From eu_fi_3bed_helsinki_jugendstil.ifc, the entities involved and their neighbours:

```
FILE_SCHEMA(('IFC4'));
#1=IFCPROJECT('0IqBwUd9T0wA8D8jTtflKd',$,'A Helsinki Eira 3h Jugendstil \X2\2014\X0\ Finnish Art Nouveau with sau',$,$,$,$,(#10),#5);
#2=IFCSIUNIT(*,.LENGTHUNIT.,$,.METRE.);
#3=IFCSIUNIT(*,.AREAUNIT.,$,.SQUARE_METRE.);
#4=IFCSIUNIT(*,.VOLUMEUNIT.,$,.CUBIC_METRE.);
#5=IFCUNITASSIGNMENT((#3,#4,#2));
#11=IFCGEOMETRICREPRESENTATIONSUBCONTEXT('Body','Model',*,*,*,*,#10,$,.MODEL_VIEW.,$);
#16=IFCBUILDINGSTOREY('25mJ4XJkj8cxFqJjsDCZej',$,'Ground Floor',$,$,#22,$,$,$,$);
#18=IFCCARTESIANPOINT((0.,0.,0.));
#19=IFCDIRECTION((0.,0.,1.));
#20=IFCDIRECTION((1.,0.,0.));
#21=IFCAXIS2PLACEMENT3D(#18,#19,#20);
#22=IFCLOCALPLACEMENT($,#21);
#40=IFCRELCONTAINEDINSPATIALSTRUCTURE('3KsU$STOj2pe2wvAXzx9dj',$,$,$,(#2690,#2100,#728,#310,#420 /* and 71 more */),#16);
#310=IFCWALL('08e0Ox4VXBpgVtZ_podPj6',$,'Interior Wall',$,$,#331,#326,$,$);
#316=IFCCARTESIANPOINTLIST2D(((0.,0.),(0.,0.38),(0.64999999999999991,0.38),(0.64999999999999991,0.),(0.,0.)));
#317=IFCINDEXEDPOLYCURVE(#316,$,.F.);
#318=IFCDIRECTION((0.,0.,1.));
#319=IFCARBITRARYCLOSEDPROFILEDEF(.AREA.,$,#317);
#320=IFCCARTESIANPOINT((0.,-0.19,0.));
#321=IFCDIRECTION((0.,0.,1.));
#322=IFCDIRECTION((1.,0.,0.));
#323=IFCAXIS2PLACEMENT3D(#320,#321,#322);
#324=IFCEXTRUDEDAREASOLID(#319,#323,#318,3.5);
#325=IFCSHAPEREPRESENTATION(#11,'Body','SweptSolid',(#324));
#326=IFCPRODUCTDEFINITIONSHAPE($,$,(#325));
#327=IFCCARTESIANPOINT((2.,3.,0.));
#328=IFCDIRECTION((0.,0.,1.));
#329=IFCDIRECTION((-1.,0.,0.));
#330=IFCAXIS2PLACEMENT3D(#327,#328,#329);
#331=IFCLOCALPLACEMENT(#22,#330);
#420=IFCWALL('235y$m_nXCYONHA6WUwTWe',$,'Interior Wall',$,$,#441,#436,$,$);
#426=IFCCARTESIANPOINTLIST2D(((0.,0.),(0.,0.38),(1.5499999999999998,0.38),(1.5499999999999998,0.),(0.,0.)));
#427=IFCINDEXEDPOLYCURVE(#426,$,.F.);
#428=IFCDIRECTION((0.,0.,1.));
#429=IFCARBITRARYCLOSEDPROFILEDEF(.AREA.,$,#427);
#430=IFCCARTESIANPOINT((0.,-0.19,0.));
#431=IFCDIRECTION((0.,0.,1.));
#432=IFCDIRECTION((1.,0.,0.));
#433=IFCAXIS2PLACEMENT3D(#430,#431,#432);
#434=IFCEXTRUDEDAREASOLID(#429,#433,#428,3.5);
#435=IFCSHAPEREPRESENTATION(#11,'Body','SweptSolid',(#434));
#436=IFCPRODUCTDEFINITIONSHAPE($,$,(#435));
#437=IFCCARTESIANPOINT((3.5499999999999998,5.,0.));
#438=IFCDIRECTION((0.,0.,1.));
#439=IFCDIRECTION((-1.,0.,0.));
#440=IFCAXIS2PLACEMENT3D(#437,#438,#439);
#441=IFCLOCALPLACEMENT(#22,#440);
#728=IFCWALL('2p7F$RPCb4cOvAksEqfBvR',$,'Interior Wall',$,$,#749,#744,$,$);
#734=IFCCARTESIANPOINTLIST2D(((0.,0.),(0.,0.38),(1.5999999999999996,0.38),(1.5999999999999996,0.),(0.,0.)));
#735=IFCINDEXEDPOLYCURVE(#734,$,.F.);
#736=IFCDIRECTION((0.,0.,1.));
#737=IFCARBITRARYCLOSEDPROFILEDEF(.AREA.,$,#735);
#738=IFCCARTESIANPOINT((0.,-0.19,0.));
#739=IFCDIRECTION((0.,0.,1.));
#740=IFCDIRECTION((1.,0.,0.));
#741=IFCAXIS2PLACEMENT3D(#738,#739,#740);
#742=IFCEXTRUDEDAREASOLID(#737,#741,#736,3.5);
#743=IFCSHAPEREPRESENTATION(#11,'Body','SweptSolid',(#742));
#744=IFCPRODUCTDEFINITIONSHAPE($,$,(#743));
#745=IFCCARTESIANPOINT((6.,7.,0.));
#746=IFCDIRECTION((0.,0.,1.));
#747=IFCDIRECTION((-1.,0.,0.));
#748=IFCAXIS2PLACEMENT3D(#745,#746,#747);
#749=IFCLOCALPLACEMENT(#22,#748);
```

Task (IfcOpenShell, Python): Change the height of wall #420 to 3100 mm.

```python
import ifcopenshell
import ifcopenshell.geom
import ifcopenshell.util.representation
import ifcopenshell.util.shape

model = ifcopenshell.open("eu_fi_3bed_helsinki_jugendstil.ifc")
settings = ifcopenshell.geom.settings()


def volume(element):
    """Net volume in cubic metres, openings subtracted."""
    shape = ifcopenshell.geom.create_shape(settings, element)
    return ifcopenshell.util.shape.get_volume(shape.geometry)


wall = model.by_id(420)
before = volume(wall)

body = ifcopenshell.util.representation.get_representation(wall, "Model", "Body")
solid = body.Items[0]
old_height = solid.Depth
solid.Depth = 3.1
after = volume(wall)

print(f"height {old_height:g} -> {solid.Depth:g}, volume {before:.3f} -> {after:.3f} m3")

model.write("eu_fi_3bed_helsinki_jugendstil_rev.ifc")
```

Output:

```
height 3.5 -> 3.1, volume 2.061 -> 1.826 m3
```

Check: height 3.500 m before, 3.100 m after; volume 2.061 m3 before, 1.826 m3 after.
